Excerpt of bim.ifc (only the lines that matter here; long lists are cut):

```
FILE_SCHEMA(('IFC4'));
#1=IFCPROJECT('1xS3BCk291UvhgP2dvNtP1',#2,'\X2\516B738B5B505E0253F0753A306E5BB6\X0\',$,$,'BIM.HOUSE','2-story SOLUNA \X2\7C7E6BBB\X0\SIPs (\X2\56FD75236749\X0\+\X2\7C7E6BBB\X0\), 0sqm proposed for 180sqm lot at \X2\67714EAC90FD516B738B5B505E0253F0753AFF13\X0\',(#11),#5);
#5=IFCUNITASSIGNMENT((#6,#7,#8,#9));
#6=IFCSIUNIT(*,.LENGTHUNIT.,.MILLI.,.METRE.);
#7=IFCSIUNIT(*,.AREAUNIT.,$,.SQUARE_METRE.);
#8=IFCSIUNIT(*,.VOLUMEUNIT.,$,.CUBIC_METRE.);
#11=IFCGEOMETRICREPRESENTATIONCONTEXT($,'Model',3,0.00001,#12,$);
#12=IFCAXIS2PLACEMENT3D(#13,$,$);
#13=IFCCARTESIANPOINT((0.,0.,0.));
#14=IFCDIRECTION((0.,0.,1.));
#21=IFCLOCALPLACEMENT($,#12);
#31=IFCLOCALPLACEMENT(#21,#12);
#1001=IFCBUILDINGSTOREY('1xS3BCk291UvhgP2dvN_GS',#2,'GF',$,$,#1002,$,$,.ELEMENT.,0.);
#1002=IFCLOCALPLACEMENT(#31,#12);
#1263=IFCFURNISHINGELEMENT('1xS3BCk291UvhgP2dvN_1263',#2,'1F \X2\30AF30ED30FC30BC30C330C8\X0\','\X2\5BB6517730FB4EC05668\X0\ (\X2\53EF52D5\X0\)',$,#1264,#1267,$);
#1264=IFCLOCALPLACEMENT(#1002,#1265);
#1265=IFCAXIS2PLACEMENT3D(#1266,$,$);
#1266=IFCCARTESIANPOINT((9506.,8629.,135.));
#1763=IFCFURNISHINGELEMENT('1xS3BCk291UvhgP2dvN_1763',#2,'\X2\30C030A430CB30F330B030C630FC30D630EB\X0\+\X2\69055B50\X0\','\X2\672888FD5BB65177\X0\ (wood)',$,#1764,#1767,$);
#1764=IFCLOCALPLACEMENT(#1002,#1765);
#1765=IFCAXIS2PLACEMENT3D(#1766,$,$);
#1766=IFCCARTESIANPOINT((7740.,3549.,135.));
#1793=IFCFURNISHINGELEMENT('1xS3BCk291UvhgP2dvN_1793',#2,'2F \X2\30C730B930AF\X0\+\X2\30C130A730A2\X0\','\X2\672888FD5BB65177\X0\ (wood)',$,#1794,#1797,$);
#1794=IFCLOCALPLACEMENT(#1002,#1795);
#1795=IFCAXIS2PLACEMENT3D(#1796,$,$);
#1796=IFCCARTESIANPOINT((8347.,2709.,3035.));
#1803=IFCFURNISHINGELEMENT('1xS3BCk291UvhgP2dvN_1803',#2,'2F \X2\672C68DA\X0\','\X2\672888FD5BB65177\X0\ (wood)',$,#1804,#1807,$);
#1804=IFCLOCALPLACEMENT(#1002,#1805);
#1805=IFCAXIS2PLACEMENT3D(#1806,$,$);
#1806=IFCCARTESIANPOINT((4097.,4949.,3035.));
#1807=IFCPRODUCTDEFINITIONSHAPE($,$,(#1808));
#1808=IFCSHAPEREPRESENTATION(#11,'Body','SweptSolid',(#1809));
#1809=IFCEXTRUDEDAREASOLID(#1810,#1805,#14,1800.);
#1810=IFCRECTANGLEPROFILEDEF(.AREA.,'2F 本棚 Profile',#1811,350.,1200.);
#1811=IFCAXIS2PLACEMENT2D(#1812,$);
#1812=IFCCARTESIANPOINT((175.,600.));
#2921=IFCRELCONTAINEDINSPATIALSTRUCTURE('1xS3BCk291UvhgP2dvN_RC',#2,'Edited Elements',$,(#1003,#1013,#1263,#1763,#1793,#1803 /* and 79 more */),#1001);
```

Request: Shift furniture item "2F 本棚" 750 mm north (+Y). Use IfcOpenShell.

```python
import ifcopenshell
import ifcopenshell.api.geometry
import ifcopenshell.util.placement
import ifcopenshell.util.unit

model = ifcopenshell.open("bim.ifc")
unit_scale = ifcopenshell.util.unit.calculate_unit_scale(model)

item = model.by_id(1803)
matrix = ifcopenshell.util.placement.get_local_placement(item.ObjectPlacement)
matrix[1, 3] += 0.75 / unit_scale
ifcopenshell.api.geometry.edit_object_placement(model, product=item, matrix=matrix, is_si=False)

print(ifcopenshell.util.placement.get_local_placement(item.ObjectPlacement).round(3) + 0.0)

model.write("bim_updated.ifc")
```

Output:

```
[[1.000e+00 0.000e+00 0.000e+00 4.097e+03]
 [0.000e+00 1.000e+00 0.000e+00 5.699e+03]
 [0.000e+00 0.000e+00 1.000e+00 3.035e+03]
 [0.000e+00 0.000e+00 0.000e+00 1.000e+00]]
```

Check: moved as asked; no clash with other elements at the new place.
